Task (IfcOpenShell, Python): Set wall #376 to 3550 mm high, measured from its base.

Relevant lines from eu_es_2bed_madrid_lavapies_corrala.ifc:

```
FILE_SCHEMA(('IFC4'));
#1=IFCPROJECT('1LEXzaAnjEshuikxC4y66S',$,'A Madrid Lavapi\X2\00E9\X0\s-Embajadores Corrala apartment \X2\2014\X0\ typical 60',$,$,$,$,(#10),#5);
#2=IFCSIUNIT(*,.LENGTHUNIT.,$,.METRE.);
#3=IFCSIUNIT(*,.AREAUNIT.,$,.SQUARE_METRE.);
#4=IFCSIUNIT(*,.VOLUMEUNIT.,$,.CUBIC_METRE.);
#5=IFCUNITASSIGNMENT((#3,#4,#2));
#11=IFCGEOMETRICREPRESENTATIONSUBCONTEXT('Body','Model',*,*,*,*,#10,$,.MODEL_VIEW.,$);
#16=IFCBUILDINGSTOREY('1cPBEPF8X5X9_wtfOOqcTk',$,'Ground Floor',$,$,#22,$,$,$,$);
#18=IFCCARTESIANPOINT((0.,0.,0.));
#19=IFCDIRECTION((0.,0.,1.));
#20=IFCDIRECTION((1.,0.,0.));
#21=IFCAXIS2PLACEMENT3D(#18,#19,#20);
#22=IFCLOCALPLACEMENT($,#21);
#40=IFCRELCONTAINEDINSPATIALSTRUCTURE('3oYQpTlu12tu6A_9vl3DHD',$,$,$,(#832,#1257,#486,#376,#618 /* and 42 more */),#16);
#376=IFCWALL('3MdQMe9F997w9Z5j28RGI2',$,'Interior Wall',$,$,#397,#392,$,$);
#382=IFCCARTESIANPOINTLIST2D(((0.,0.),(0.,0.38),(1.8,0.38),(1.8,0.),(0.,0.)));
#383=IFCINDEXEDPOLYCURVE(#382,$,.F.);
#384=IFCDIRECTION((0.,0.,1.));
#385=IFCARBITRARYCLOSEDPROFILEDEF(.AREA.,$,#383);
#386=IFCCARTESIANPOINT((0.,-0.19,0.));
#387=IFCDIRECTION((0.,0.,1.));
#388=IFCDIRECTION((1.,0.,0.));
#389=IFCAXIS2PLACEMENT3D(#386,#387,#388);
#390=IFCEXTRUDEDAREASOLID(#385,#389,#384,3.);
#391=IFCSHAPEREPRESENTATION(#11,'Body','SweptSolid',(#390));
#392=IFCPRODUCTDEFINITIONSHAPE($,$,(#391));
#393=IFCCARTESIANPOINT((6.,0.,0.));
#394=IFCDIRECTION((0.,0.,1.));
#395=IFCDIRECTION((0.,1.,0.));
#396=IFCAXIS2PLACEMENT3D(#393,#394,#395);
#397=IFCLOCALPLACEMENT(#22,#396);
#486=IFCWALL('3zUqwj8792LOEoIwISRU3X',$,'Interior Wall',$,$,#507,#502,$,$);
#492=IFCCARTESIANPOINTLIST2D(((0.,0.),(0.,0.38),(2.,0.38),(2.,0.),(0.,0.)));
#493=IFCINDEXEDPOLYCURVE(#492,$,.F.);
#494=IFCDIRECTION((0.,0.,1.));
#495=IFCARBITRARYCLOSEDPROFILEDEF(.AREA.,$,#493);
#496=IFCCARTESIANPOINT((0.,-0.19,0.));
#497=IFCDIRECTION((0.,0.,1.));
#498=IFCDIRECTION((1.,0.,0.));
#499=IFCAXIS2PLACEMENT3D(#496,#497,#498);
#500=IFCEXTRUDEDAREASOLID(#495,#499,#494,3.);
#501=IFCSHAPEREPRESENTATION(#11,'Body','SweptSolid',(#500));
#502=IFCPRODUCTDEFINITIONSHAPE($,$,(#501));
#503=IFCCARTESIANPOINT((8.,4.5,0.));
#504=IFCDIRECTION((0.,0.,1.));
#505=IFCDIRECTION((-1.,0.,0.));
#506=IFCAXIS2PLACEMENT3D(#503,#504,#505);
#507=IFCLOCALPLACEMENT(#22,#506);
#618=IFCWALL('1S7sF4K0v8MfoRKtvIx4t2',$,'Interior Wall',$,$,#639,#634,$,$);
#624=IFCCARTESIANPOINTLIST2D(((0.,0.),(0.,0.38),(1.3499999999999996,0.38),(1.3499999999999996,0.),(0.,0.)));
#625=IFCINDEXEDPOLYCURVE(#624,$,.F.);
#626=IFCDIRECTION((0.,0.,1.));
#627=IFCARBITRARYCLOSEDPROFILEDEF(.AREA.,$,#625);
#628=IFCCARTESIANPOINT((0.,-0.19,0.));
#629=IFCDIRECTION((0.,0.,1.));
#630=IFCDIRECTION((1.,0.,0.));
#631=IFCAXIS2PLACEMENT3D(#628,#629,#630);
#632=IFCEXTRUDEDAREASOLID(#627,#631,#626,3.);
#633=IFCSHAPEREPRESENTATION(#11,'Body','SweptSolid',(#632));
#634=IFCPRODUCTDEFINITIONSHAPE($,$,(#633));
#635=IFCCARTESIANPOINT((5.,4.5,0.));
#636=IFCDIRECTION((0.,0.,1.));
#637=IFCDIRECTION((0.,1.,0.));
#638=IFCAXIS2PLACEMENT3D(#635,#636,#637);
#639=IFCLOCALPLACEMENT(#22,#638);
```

```python
import ifcopenshell
import ifcopenshell.geom
import ifcopenshell.util.representation
import ifcopenshell.util.shape
import ifcopenshell.util.unit

model = ifcopenshell.open("eu_es_2bed_madrid_lavapies_corrala.ifc")
unit_scale = ifcopenshell.util.unit.calculate_unit_scale(model)
settings = ifcopenshell.geom.settings()


def volume(element):
    """Net volume in cubic metres, openings subtracted."""
    shape = ifcopenshell.geom.create_shape(settings, element)
    return ifcopenshell.util.shape.get_volume(shape.geometry)


wall = model.by_guid("3MdQMe9F997w9Z5j28RGI2")
before = volume(wall)

body = ifcopenshell.util.representation.get_representation(wall, "Model", "Body")
solid = body.Items[0]
old_height = solid.Depth
solid.Depth = 3.55 / unit_scale
after = volume(wall)

print(f"height {old_height:g} -> {solid.Depth:g}, volume {before:.3f} -> {after:.3f} m3")

model.write("eu_es_2bed_madrid_lavapies_corrala_v2.ifc")
```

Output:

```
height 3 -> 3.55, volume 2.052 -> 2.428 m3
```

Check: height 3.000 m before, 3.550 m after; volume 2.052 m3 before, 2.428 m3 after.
